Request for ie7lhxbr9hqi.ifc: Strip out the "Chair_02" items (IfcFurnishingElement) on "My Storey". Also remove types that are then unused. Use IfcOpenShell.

First a look at what the model holds.

```python
import ifcopenshell
import ifcopenshell.util.element

model = ifcopenshell.open("ie7lhxbr9hqi.ifc")
print(model.schema)
storey = next(s for s in model.by_type("IfcBuildingStorey") if s.Name == "My Storey")
furniture = [e for e in ifcopenshell.util.element.get_decomposition(storey) if e.is_a("IfcFurnishingElement")]
seen = {}
for e in furniture:
    element_type = ifcopenshell.util.element.get_type(e)
    name = element_type.Name if element_type not in (None, e) else None
    seen[name] = seen.get(name, 0) + 1
for name, count in sorted(seen.items(), key=str):
    print(count, "x", name)
```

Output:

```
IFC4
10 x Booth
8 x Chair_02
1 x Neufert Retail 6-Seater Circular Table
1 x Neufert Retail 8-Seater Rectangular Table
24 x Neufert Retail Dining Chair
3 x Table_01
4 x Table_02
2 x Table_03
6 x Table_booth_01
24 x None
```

```python
import ifcopenshell
import ifcopenshell.api.root
import ifcopenshell.util.element

model = ifcopenshell.open("ie7lhxbr9hqi.ifc")

storey = next(s for s in model.by_type("IfcBuildingStorey") if s.Name == "My Storey")
furniture = [e for e in ifcopenshell.util.element.get_decomposition(storey) if e.is_a("IfcFurnishingElement")]
targets = [e for e in furniture if (t := ifcopenshell.util.element.get_type(e)) not in (None, e) and t.Name == "Chair_02"]
types = {ifcopenshell.util.element.get_type(e) for e in targets} - {None, *targets}

for e in targets:
    ifcopenshell.api.root.remove_product(model, product=e)
print(len(targets), "removed")

unused = [t for t in types if not ifcopenshell.util.element.get_types(t)]
for t in unused:
    ifcopenshell.api.root.remove_product(model, product=t)
print(len(unused), "unused types removed")

model.write("ie7lhxbr9hqi_updated.ifc")
```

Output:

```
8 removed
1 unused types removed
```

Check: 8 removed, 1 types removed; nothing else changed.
